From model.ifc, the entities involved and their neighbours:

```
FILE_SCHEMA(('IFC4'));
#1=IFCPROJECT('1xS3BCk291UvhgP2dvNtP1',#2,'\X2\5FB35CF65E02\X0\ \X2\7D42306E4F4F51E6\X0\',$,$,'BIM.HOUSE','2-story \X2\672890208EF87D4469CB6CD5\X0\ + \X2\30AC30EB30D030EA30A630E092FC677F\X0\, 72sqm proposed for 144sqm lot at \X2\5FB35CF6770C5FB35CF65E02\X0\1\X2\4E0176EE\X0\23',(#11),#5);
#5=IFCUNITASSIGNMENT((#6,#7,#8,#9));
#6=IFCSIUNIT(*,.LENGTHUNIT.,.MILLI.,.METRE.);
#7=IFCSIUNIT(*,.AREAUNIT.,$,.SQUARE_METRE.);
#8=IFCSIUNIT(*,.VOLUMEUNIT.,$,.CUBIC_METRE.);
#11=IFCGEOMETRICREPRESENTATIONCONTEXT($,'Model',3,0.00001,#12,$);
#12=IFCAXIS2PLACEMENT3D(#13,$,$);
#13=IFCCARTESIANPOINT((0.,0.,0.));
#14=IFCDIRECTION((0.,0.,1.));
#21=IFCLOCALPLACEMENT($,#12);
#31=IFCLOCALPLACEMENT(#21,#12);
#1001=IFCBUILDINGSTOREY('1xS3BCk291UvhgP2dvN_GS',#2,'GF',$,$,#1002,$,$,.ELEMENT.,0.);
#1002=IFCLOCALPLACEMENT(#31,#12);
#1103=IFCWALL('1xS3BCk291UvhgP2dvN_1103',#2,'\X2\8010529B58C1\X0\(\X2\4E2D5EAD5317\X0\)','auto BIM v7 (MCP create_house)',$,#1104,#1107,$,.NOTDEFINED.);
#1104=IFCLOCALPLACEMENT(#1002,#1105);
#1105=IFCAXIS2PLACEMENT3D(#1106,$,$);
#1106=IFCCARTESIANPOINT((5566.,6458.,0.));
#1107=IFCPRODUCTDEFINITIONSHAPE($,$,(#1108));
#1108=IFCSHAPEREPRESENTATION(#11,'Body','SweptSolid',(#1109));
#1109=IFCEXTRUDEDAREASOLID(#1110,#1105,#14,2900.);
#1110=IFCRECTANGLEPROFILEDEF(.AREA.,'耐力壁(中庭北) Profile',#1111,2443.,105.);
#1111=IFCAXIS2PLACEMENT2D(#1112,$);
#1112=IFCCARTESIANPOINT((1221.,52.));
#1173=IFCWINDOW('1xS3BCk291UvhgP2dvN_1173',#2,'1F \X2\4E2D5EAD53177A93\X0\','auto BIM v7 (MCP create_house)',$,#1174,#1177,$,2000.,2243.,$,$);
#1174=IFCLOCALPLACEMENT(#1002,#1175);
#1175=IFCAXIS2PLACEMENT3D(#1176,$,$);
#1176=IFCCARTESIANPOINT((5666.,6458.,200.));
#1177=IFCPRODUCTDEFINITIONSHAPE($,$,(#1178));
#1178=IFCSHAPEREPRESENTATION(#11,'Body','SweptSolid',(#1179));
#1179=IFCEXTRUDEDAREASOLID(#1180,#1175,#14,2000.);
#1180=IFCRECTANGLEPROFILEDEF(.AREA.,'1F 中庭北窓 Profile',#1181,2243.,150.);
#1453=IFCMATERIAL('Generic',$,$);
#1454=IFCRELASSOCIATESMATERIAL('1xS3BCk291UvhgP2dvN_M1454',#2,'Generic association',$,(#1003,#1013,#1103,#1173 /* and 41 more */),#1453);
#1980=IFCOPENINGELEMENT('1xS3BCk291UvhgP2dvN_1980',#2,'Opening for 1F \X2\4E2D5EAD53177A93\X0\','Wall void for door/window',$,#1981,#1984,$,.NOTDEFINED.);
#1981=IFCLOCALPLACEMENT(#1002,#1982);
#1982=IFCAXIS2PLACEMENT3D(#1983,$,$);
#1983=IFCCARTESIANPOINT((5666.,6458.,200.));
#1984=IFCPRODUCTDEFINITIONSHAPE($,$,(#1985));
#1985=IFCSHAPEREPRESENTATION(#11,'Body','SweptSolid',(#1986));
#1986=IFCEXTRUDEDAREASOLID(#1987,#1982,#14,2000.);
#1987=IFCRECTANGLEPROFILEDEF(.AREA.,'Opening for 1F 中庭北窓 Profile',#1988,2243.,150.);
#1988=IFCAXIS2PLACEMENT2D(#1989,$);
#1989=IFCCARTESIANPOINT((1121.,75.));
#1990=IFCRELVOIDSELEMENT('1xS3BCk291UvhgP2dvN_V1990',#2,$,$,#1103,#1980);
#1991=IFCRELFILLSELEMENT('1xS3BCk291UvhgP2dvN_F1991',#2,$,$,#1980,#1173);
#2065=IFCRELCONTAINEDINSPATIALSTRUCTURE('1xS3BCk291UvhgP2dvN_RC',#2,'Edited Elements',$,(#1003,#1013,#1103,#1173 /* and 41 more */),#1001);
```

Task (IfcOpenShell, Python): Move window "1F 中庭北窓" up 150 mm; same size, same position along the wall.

```python
import numpy as np
import ifcopenshell
import ifcopenshell.api.geometry
import ifcopenshell.util.placement
import ifcopenshell.util.unit

model = ifcopenshell.open("model.ifc")
unit_scale = ifcopenshell.util.unit.calculate_unit_scale(model)

window = model.by_guid("1xS3BCk291UvhgP2dvN_1173")
opening = window.FillsVoids[0].RelatingOpeningElement
dz = 0.15 / unit_scale

shift = np.array([0.0, 0.0, dz])
# The window is not placed relative to its opening, so move both.
for product in (opening, window):
    matrix = ifcopenshell.util.placement.get_local_placement(product.ObjectPlacement)
    matrix[:3, 3] += shift
    ifcopenshell.api.geometry.edit_object_placement(model, product=product, matrix=matrix, is_si=False)

print(f"moved by {dz * unit_scale:+.3f} m")

model.write("model_v2.ifc")
```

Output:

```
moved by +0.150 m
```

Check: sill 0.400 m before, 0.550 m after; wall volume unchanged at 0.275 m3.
